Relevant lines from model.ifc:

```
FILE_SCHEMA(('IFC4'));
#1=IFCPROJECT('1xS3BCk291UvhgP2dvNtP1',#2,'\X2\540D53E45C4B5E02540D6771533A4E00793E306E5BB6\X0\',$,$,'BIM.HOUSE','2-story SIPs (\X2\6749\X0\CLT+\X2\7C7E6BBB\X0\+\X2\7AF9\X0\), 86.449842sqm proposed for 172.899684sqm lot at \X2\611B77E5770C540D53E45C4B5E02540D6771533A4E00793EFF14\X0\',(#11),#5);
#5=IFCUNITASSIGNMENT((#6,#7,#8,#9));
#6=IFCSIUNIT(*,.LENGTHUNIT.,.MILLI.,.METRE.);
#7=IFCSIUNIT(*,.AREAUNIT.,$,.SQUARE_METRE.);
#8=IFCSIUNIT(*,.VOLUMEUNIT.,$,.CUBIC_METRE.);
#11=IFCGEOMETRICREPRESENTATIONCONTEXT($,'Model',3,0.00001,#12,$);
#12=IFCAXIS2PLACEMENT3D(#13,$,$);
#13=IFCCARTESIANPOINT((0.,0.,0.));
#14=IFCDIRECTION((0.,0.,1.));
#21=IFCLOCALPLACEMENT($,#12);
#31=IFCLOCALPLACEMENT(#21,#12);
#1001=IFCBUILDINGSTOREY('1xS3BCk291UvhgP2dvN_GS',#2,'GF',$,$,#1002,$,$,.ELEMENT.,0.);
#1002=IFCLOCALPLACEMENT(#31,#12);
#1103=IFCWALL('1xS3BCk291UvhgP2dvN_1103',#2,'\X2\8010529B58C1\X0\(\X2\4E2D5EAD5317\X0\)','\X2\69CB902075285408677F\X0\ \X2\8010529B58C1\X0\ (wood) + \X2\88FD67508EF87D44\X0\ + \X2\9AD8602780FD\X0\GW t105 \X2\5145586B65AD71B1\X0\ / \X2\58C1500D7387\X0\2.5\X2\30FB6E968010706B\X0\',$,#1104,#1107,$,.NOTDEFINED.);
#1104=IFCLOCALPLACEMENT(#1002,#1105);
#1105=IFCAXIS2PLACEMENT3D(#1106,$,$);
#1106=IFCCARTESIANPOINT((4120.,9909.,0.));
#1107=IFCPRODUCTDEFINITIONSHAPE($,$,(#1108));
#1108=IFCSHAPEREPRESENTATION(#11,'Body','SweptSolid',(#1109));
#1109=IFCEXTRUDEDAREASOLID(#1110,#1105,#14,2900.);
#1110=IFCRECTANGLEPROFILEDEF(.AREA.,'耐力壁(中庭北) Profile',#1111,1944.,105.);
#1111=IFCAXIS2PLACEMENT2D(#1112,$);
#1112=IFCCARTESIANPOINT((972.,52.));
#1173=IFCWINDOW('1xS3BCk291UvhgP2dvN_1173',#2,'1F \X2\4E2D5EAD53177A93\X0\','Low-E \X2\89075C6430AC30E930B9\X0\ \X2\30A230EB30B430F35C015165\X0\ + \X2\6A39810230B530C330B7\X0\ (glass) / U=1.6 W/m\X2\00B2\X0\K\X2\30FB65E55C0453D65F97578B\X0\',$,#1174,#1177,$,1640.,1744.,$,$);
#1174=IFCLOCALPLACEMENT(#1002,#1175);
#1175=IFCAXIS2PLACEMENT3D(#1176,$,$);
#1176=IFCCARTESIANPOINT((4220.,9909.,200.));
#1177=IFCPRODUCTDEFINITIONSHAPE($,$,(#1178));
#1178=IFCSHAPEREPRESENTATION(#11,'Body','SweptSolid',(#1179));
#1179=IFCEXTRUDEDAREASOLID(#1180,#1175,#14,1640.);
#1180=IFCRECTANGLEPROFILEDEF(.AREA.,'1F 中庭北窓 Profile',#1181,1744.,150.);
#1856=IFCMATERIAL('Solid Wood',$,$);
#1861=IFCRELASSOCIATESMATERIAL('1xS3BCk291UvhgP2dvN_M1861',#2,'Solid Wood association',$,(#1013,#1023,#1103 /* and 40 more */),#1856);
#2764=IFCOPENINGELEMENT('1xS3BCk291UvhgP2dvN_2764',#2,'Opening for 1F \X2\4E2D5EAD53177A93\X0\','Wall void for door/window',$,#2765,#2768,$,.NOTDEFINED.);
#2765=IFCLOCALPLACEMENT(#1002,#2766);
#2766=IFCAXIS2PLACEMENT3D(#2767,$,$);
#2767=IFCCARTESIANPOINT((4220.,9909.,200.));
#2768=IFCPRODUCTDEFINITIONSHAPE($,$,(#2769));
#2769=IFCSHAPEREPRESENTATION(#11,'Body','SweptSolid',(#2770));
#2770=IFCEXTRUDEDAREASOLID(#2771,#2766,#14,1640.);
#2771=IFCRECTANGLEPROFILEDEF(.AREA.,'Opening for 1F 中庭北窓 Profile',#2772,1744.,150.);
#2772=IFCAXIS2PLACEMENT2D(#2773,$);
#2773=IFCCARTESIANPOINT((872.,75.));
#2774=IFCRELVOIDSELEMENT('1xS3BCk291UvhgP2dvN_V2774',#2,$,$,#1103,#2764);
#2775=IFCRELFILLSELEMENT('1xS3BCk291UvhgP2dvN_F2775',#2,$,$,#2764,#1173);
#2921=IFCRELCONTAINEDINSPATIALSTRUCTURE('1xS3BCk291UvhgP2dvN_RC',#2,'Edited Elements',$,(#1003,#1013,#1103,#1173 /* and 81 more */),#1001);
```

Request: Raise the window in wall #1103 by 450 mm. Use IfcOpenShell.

```python
import numpy as np
import ifcopenshell
import ifcopenshell.api.geometry
import ifcopenshell.util.placement
import ifcopenshell.util.unit

model = ifcopenshell.open("model.ifc")
unit_scale = ifcopenshell.util.unit.calculate_unit_scale(model)

window = model.by_guid("1xS3BCk291UvhgP2dvN_1173")
opening = window.FillsVoids[0].RelatingOpeningElement
dz = 0.45 / unit_scale

shift = np.array([0.0, 0.0, dz])
# The window is not placed relative to its opening, so move both.
for product in (opening, window):
    matrix = ifcopenshell.util.placement.get_local_placement(product.ObjectPlacement)
    matrix[:3, 3] += shift
    ifcopenshell.api.geometry.edit_object_placement(model, product=product, matrix=matrix, is_si=False)

print(f"moved by {dz * unit_scale:+.3f} m")

model.write("model_rev.ifc")
```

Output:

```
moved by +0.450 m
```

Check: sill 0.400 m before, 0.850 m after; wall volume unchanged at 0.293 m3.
